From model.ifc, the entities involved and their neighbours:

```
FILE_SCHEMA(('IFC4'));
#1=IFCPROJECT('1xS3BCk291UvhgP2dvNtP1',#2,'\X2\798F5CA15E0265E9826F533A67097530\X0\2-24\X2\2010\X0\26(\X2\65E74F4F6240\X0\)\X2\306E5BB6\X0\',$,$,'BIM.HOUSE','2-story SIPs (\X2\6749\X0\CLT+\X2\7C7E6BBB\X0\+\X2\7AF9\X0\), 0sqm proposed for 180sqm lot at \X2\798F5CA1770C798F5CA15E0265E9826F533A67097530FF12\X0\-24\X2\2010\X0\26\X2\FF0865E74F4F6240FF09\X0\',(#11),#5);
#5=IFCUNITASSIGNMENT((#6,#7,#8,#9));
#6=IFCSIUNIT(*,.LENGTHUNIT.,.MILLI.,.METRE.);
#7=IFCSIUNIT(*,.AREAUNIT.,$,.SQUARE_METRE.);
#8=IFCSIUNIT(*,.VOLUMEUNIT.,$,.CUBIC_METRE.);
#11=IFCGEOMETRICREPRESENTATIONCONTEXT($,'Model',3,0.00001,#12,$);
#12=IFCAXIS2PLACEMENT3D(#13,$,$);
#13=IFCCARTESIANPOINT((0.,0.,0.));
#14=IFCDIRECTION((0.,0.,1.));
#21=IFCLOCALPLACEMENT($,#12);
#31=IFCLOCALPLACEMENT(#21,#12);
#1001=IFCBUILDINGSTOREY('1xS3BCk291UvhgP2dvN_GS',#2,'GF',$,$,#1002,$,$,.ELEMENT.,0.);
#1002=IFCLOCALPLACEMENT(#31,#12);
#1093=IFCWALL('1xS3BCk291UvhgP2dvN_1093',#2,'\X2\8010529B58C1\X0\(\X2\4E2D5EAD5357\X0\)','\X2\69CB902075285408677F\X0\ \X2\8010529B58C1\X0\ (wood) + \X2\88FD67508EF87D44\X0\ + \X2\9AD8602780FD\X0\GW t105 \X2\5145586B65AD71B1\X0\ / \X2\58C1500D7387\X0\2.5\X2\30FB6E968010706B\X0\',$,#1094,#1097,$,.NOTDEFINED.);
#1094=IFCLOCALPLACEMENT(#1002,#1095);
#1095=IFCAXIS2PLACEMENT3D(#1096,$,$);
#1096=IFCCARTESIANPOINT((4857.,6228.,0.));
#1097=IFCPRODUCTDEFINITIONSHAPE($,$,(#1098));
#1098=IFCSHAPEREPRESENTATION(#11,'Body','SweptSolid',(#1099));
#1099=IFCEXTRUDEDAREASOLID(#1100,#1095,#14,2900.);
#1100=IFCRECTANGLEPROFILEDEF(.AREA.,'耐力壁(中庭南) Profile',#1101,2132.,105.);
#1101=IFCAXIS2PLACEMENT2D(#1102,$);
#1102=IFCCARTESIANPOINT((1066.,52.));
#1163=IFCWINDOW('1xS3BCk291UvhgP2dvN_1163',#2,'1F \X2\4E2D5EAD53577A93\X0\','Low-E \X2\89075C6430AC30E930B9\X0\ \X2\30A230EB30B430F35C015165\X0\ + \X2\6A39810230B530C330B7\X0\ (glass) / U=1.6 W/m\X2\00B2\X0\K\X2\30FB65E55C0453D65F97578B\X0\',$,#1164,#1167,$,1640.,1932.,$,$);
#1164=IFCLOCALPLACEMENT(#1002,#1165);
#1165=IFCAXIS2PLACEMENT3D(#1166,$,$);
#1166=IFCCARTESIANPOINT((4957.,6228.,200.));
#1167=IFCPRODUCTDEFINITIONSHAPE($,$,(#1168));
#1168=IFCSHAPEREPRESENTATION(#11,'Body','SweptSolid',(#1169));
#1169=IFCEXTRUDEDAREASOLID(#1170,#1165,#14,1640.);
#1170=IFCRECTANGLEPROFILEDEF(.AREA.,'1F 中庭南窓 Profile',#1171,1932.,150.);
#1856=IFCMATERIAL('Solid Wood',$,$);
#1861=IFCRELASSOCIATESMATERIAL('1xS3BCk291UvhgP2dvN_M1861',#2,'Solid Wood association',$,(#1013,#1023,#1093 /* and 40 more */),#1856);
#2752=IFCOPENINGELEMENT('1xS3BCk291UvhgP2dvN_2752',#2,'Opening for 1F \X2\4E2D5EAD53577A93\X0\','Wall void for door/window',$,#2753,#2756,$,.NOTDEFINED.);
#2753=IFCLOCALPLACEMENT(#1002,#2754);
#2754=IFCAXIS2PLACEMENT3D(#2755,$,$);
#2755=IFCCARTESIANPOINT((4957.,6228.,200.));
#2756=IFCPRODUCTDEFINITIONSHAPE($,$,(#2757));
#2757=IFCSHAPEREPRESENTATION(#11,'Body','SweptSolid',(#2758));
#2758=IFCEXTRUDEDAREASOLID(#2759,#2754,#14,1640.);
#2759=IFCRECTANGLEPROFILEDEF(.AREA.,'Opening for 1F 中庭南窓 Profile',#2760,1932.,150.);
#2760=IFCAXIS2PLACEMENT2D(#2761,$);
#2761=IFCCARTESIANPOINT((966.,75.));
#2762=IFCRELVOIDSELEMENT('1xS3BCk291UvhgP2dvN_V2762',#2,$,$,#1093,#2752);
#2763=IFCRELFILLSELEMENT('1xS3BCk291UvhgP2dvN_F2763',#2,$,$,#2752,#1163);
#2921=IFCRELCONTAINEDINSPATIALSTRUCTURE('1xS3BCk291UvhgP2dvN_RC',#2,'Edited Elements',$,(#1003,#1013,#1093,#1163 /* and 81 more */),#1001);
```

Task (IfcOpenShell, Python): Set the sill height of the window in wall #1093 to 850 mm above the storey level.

```python
import numpy as np
import ifcopenshell
import ifcopenshell.api.geometry
import ifcopenshell.geom
import ifcopenshell.util.element
import ifcopenshell.util.placement
import ifcopenshell.util.shape
import ifcopenshell.util.unit

model = ifcopenshell.open("model.ifc")
unit_scale = ifcopenshell.util.unit.calculate_unit_scale(model)

window = model.by_id(1163)
opening = window.FillsVoids[0].RelatingOpeningElement
storey = ifcopenshell.util.element.get_container(window, ifc_class="IfcBuildingStorey")
level = ifcopenshell.util.placement.get_local_placement(storey.ObjectPlacement)[2, 3]

# The opening's origin need not be at the sill, so measure its lowest point.
shape = ifcopenshell.geom.create_shape(ifcopenshell.geom.settings(), opening)
bottom = ifcopenshell.util.shape.get_shape_bottom_elevation(shape, shape.geometry) / unit_scale
dz = level + 0.85 / unit_scale - bottom

shift = np.array([0.0, 0.0, dz])
# The window is not placed relative to its opening, so move both.
for product in (opening, window):
    matrix = ifcopenshell.util.placement.get_local_placement(product.ObjectPlacement)
    matrix[:3, 3] += shift
    ifcopenshell.api.geometry.edit_object_placement(model, product=product, matrix=matrix, is_si=False)

print(f"moved by {dz * unit_scale:+.3f} m")

model.write("model_edited.ifc")
```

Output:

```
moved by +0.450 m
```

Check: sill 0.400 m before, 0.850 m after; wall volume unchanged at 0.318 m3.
